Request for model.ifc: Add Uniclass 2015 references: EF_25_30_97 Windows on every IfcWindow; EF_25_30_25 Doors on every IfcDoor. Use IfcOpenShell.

First a look at what the model holds.

```python
import ifcopenshell

model = ifcopenshell.open("model.ifc")
print(model.schema)
print("classifications:", [c.Name for c in model.by_type("IfcClassification")])
for ifc_class in ("IfcDoor", "IfcRoof", "IfcStair", "IfcWall", "IfcWindow"):
    print(ifc_class, len(model.by_type(ifc_class)))
```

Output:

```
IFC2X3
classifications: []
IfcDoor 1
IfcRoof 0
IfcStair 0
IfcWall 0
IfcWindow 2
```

```python
import ifcopenshell
import ifcopenshell.api.classification

model = ifcopenshell.open("model.ifc")

# IFC2X3 requires Source and Edition and has no link from the project to the system.
system = model.create_entity("IfcClassification", Source="NBS", Edition="2015", Name="Uniclass 2015")

codes = {
    "IfcWindow": ("EF_25_30_97", "Windows"),
    "IfcDoor": ("EF_25_30_25", "Doors"),
}
for ifc_class, (code, name) in codes.items():
    products = model.by_type(ifc_class)
    ifcopenshell.api.classification.add_reference(
        model, products=products, classification=system, identification=code, name=name
    )
    print(code, len(products))

model.write("model-out.ifc")
```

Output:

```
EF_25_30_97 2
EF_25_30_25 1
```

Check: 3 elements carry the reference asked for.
